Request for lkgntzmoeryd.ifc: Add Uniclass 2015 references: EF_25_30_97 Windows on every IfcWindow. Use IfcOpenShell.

First a look at what the model holds.

```python
import ifcopenshell

model = ifcopenshell.open("lkgntzmoeryd.ifc")
print(model.schema)
print("classifications:", [c.Name for c in model.by_type("IfcClassification")])
for ifc_class in ("IfcDoor", "IfcRoof", "IfcStair", "IfcWall", "IfcWindow"):
    print(ifc_class, len(model.by_type(ifc_class)))
```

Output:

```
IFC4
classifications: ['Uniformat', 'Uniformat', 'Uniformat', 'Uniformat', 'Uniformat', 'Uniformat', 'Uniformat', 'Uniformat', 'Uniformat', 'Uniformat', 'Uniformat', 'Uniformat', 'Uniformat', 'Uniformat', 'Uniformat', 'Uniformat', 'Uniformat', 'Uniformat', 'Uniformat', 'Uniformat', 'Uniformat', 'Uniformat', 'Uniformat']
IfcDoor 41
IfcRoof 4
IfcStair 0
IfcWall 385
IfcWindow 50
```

```python
import ifcopenshell
import ifcopenshell.api.classification

model = ifcopenshell.open("lkgntzmoeryd.ifc")

system = ifcopenshell.api.classification.add_classification(model, classification="Uniclass 2015")

codes = {
    "IfcWindow": ("EF_25_30_97", "Windows"),
}
for ifc_class, (code, name) in codes.items():
    products = model.by_type(ifc_class)
    ifcopenshell.api.classification.add_reference(
        model, products=products, classification=system, identification=code, name=name
    )
    print(code, len(products))

model.write("lkgntzmoeryd-out.ifc")
```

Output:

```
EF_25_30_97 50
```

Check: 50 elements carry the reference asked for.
